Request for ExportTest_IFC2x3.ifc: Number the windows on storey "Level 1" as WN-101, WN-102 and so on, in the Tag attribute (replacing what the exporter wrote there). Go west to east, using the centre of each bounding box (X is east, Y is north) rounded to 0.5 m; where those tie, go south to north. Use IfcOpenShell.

First a look at what the model holds.

```python
import ifcopenshell
import ifcopenshell.util.element
import ifcopenshell.util.placement

model = ifcopenshell.open("ExportTest_IFC2x3.ifc")
print(model.schema)
storey = next(s for s in model.by_type("IfcBuildingStorey") if s.Name == "Level 1")
windows = [e for e in ifcopenshell.util.element.get_decomposition(storey) if e.is_a("IfcWindow")]
for e in sorted(windows, key=lambda e: e.id()):
    origin = ifcopenshell.util.placement.get_local_placement(e.ObjectPlacement)[:3, 3]
    print(e.id(), e.Tag, e.Name, origin.round(2) + 0.0, sep=" | ")
```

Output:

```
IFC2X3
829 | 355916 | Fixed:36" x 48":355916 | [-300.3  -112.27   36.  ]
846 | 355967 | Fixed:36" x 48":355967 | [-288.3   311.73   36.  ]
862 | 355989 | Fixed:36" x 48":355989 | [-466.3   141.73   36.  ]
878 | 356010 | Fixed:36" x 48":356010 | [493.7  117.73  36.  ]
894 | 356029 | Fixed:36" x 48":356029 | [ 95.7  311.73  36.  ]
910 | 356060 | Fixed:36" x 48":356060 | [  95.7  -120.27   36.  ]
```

```python
import ifcopenshell
import ifcopenshell.geom
import ifcopenshell.util.element
import ifcopenshell.util.shape

model = ifcopenshell.open("ExportTest_IFC2x3.ifc")
settings = ifcopenshell.geom.settings()
settings.set("use-world-coords", True)


def centre(element):
    shape = ifcopenshell.geom.create_shape(settings, element)
    return ifcopenshell.util.shape.get_bbox_centroid(shape.geometry)


storey = next(s for s in model.by_type("IfcBuildingStorey") if s.Name == "Level 1")
windows = [e for e in ifcopenshell.util.element.get_decomposition(storey) if e.is_a("IfcWindow")]

# Insertion points can sit at a corner or the storey origin, so sort by the geometry (in metres).
centres = {e: centre(e) for e in windows}
windows.sort(key=lambda e: (round(centres[e][0] / 0.5), centres[e][1]))

for i, e in enumerate(windows, start=1):
    number = f"WN-1{i:02d}"
    e.Tag = number
    print(e.id(), number)

model.write("ExportTest_IFC2x3_edited.ifc")
```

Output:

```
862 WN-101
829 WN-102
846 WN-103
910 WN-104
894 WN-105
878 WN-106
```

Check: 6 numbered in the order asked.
